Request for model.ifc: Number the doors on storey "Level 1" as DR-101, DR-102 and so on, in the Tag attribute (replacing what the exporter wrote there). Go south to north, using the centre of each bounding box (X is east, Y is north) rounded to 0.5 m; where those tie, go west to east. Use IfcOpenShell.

First a look at what the model holds.

```python
import ifcopenshell
import ifcopenshell.util.element
import ifcopenshell.util.placement

model = ifcopenshell.open("model.ifc")
print(model.schema)
storey = next(s for s in model.by_type("IfcBuildingStorey") if s.Name == "Level 1")
doors = [e for e in ifcopenshell.util.element.get_decomposition(storey) if e.is_a("IfcDoor")]
for e in sorted(doors, key=lambda e: e.id()):
    origin = ifcopenshell.util.placement.get_local_placement(e.ObjectPlacement)[:3, 3]
    print(e.id(), e.Tag, e.Name, origin.round(2) + 0.0, sep=" | ")
```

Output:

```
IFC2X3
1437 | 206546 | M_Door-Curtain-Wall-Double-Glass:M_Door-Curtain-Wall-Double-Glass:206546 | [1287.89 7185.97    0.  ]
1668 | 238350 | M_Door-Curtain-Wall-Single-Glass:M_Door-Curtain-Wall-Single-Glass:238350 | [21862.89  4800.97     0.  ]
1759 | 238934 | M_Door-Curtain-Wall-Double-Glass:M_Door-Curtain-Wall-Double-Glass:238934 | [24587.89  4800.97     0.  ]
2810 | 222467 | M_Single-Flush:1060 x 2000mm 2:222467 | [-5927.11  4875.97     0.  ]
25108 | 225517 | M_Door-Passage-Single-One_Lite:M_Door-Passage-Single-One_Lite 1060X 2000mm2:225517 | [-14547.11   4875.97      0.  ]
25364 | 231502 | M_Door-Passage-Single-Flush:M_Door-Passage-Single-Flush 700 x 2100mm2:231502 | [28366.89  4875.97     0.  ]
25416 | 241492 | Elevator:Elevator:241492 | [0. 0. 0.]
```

```python
import ifcopenshell
import ifcopenshell.geom
import ifcopenshell.util.element
import ifcopenshell.util.shape

model = ifcopenshell.open("model.ifc")
settings = ifcopenshell.geom.settings()
settings.set("use-world-coords", True)


def centre(element):
    shape = ifcopenshell.geom.create_shape(settings, element)
    return ifcopenshell.util.shape.get_bbox_centroid(shape.geometry)


storey = next(s for s in model.by_type("IfcBuildingStorey") if s.Name == "Level 1")
doors = [e for e in ifcopenshell.util.element.get_decomposition(storey) if e.is_a("IfcDoor")]

# Insertion points can sit at a corner or the storey origin, so sort by the geometry (in metres).
centres = {e: centre(e) for e in doors}
doors.sort(key=lambda e: (round(centres[e][1] / 0.5), centres[e][0]))

for i, e in enumerate(doors, start=1):
    number = f"DR-1{i:02d}"
    e.Tag = number
    print(e.id(), number)

model.write("model-out.ifc")
```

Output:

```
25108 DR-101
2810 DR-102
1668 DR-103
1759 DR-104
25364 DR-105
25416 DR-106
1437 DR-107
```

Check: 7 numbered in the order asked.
